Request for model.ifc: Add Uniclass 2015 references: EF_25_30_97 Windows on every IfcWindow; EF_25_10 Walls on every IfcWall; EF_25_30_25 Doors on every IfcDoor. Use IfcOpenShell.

First a look at what the model holds.

```python
import ifcopenshell

model = ifcopenshell.open("model.ifc")
print(model.schema)
print("classifications:", [c.Name for c in model.by_type("IfcClassification")])
for ifc_class in ("IfcDoor", "IfcRoof", "IfcStair", "IfcWall", "IfcWindow"):
    print(ifc_class, len(model.by_type(ifc_class)))
```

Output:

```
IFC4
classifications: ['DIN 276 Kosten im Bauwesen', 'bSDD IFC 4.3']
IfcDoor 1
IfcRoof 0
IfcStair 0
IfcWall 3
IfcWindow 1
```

```python
import ifcopenshell
import ifcopenshell.api.classification

model = ifcopenshell.open("model.ifc")

system = ifcopenshell.api.classification.add_classification(model, classification="Uniclass 2015")

codes = {
    "IfcWindow": ("EF_25_30_97", "Windows"),
    "IfcWall": ("EF_25_10", "Walls"),
    "IfcDoor": ("EF_25_30_25", "Doors"),
}
for ifc_class, (code, name) in codes.items():
    products = model.by_type(ifc_class)
    ifcopenshell.api.classification.add_reference(
        model, products=products, classification=system, identification=code, name=name
    )
    print(code, len(products))

model.write("model_v2.ifc")
```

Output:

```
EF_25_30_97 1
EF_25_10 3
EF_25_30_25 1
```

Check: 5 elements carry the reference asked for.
